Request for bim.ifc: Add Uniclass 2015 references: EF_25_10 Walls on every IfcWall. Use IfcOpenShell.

First a look at what the model holds.

```python
import ifcopenshell

model = ifcopenshell.open("bim.ifc")
print(model.schema)
print("classifications:", [c.Name for c in model.by_type("IfcClassification")])
for ifc_class in ("IfcDoor", "IfcRoof", "IfcStair", "IfcWall", "IfcWindow"):
    print(ifc_class, len(model.by_type(ifc_class)))
```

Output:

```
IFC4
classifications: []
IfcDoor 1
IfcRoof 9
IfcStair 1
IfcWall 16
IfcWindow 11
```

```python
import ifcopenshell
import ifcopenshell.api.classification

model = ifcopenshell.open("bim.ifc")

system = ifcopenshell.api.classification.add_classification(model, classification="Uniclass 2015")

codes = {
    "IfcWall": ("EF_25_10", "Walls"),
}
for ifc_class, (code, name) in codes.items():
    products = model.by_type(ifc_class)
    ifcopenshell.api.classification.add_reference(
        model, products=products, classification=system, identification=code, name=name
    )
    print(code, len(products))

model.write("bim-out.ifc")
```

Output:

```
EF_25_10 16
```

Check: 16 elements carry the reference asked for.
